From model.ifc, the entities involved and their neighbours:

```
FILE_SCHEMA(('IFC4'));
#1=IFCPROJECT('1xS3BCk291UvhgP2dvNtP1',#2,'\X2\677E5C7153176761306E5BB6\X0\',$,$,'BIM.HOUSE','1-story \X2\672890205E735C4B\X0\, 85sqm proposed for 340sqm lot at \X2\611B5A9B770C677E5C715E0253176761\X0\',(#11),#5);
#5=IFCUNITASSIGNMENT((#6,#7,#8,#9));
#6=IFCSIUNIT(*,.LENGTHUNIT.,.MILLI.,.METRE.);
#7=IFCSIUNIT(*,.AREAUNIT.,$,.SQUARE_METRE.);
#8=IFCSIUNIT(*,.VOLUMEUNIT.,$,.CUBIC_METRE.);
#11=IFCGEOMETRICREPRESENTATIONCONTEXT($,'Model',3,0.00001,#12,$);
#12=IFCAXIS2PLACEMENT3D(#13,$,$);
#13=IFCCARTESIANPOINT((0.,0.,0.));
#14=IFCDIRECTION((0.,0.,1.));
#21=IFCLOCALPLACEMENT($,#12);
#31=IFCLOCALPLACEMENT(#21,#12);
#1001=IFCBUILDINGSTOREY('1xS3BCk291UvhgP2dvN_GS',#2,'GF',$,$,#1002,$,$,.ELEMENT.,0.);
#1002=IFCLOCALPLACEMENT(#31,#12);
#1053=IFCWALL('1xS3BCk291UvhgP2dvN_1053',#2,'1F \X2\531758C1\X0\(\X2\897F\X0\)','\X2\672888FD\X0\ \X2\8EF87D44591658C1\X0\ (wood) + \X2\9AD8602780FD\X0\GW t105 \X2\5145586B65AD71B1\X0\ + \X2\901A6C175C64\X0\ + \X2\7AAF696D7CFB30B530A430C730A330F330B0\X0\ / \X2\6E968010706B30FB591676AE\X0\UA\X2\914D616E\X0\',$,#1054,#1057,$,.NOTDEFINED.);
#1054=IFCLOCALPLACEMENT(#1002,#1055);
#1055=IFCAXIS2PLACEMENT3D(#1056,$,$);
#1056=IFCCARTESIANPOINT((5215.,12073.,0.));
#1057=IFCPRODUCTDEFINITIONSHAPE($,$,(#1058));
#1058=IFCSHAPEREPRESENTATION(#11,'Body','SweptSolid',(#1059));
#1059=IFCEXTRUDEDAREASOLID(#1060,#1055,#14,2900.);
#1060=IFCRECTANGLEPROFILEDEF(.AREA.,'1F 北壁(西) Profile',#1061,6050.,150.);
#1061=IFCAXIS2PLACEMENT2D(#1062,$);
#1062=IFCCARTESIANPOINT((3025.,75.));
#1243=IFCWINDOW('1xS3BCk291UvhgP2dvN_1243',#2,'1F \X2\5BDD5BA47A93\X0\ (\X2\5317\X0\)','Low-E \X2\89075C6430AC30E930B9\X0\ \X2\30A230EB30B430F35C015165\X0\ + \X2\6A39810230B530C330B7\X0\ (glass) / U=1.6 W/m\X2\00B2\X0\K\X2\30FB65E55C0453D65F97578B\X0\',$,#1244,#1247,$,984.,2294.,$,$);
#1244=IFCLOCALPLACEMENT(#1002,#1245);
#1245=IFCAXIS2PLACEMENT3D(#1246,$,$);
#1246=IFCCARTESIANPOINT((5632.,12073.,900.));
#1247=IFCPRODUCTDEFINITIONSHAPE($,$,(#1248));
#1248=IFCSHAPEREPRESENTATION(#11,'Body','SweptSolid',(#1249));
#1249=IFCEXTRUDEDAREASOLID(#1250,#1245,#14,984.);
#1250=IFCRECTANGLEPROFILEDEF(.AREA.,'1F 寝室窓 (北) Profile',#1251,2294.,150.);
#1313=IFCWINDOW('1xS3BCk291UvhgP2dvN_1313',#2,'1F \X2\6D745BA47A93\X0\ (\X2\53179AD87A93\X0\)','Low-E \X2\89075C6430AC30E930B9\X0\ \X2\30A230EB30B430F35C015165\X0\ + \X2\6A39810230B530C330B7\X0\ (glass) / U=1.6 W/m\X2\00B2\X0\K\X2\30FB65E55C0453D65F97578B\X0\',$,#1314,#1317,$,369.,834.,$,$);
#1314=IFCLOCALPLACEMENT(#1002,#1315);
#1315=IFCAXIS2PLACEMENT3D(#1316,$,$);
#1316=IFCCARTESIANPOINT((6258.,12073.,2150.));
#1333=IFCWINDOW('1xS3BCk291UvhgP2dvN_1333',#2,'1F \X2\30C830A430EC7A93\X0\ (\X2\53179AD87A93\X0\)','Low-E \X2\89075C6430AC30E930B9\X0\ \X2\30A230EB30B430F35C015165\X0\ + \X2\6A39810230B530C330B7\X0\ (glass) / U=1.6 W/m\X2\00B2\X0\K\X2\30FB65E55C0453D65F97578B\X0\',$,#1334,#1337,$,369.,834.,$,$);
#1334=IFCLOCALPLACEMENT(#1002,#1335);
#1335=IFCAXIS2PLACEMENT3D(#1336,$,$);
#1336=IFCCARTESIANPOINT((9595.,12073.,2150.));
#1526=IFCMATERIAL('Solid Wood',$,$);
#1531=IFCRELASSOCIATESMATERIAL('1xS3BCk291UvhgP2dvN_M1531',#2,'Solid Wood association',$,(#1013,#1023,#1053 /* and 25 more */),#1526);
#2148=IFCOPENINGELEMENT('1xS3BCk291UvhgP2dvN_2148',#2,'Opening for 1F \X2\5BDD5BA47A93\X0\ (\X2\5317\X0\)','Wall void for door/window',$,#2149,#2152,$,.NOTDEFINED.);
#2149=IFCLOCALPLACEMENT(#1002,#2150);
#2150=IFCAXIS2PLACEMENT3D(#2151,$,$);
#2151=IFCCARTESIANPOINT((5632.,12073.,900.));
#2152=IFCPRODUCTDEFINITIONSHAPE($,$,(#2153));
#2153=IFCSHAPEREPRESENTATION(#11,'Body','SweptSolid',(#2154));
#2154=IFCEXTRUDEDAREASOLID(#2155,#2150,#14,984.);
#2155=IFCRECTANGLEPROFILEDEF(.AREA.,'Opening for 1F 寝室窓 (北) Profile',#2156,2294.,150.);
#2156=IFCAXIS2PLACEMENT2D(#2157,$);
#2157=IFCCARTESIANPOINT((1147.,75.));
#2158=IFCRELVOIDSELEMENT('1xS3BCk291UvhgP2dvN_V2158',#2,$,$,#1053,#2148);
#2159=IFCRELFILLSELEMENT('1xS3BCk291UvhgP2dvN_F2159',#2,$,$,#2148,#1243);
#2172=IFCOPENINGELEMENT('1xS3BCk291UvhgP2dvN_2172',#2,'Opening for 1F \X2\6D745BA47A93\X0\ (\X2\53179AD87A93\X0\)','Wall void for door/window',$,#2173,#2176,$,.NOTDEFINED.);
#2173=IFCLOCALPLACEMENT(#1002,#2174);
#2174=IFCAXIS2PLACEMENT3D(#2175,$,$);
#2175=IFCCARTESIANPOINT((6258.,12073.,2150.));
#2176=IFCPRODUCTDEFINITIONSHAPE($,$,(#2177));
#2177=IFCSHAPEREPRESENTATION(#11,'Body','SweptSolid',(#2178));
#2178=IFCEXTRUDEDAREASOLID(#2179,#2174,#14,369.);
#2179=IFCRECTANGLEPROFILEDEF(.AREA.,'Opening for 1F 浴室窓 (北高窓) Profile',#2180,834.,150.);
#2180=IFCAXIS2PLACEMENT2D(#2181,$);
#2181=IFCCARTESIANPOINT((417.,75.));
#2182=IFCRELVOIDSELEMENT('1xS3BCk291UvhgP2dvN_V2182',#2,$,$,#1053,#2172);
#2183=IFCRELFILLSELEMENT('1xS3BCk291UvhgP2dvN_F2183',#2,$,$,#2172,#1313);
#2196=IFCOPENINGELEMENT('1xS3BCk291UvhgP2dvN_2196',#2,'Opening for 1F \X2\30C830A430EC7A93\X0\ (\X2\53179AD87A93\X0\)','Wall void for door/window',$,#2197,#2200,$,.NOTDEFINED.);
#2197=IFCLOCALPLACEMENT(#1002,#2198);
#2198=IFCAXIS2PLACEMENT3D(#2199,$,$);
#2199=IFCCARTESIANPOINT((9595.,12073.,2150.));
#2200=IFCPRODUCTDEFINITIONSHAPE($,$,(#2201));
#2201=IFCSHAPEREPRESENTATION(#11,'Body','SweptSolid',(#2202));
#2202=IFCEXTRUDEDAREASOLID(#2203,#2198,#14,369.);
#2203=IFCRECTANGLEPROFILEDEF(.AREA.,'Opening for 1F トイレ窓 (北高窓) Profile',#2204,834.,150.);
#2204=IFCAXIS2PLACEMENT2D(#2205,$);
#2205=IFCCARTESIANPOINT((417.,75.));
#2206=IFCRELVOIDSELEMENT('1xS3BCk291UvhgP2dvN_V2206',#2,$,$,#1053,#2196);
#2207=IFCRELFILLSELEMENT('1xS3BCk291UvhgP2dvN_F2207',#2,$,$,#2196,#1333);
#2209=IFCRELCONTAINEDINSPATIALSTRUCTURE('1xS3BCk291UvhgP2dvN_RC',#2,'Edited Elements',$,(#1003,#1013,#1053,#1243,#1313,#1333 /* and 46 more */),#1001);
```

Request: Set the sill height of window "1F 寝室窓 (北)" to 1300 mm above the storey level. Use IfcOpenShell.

```python
import numpy as np
import ifcopenshell
import ifcopenshell.api.geometry
import ifcopenshell.geom
import ifcopenshell.util.element
import ifcopenshell.util.placement
import ifcopenshell.util.shape
import ifcopenshell.util.unit

model = ifcopenshell.open("model.ifc")
unit_scale = ifcopenshell.util.unit.calculate_unit_scale(model)

window = model.by_id(1243)
opening = window.FillsVoids[0].RelatingOpeningElement
storey = ifcopenshell.util.element.get_container(window, ifc_class="IfcBuildingStorey")
level = ifcopenshell.util.placement.get_local_placement(storey.ObjectPlacement)[2, 3]

# The opening's origin need not be at the sill, so measure its lowest point.
shape = ifcopenshell.geom.create_shape(ifcopenshell.geom.settings(), opening)
bottom = ifcopenshell.util.shape.get_shape_bottom_elevation(shape, shape.geometry) / unit_scale
dz = level + 1.3 / unit_scale - bottom

shift = np.array([0.0, 0.0, dz])
# The window is not placed relative to its opening, so move both.
for product in (opening, window):
    matrix = ifcopenshell.util.placement.get_local_placement(product.ObjectPlacement)
    matrix[:3, 3] += shift
    ifcopenshell.api.geometry.edit_object_placement(model, product=product, matrix=matrix, is_si=False)

print(f"moved by {dz * unit_scale:+.3f} m")

model.write("model_rev.ifc")
```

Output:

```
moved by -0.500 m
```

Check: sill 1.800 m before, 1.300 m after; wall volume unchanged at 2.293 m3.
